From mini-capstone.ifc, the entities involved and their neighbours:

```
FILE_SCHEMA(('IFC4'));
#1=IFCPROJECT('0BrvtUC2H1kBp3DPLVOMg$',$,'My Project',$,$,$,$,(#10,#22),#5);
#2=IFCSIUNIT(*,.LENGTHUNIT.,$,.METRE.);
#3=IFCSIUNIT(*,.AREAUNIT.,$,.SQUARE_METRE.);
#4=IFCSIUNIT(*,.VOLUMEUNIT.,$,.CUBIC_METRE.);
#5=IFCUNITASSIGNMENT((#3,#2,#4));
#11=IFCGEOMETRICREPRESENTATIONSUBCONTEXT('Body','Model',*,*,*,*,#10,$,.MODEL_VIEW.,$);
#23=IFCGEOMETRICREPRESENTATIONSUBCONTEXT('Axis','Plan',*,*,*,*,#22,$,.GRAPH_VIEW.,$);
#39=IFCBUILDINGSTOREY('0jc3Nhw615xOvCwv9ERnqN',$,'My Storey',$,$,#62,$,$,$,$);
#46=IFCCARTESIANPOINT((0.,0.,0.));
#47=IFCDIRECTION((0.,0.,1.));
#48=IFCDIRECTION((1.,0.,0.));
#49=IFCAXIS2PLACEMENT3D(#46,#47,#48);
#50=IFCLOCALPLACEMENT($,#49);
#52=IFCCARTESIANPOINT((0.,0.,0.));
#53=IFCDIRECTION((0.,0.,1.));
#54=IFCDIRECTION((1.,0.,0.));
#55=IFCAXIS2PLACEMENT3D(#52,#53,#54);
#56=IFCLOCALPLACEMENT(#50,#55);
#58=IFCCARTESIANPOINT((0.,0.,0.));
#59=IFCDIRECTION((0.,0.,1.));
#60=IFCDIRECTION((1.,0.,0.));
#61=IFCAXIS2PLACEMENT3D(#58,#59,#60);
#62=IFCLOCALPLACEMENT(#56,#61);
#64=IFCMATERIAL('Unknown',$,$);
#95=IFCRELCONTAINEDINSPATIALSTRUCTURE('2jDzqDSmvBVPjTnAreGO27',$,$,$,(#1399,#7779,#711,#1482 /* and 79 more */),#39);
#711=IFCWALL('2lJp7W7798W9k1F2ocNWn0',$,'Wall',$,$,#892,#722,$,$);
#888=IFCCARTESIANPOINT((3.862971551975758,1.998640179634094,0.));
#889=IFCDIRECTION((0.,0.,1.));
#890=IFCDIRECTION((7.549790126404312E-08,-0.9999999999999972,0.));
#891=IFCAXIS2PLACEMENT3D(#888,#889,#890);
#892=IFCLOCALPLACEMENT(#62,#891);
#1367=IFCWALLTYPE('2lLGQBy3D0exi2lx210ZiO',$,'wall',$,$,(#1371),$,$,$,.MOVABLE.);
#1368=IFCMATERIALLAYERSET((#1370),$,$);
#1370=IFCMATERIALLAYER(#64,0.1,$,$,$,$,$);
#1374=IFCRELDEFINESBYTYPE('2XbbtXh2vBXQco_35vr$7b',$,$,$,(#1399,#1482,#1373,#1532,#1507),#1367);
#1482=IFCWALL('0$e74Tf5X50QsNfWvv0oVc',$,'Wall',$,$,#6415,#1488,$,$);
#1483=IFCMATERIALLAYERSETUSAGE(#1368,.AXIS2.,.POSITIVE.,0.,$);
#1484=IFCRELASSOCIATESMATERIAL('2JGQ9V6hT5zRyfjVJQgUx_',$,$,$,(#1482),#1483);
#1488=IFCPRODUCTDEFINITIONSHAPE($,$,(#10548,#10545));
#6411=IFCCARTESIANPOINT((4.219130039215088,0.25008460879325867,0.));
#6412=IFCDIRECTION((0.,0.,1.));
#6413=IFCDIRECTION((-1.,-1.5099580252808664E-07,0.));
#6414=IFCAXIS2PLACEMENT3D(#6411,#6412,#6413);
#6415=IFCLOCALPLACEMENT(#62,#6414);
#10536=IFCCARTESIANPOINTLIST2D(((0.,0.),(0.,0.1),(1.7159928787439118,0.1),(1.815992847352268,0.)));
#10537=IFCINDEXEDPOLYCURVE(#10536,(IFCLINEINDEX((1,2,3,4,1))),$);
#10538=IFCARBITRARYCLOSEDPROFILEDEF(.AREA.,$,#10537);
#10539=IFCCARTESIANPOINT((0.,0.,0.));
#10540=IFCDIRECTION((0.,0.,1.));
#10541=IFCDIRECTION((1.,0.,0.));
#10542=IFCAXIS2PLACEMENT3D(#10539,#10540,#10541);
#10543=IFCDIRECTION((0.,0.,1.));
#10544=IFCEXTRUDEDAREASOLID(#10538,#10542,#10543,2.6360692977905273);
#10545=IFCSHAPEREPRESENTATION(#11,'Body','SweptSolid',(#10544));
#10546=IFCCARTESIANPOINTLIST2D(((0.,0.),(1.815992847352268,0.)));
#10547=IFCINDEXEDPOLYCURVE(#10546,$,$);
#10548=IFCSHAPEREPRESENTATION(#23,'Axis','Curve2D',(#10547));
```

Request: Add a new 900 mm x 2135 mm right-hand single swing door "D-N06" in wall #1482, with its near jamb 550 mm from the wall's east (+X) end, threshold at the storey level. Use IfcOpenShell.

```python
import numpy as np
import ifcopenshell
import ifcopenshell.api.feature
import ifcopenshell.api.geometry
import ifcopenshell.api.root
import ifcopenshell.api.spatial
import ifcopenshell.geom
import ifcopenshell.util.element
import ifcopenshell.util.placement
import ifcopenshell.util.representation
import ifcopenshell.util.shape
import ifcopenshell.util.unit

model = ifcopenshell.open("mini-capstone.ifc")
unit_scale = ifcopenshell.util.unit.calculate_unit_scale(model)
settings = ifcopenshell.geom.settings()


def volume(element):
    """Net volume in cubic metres, openings subtracted."""
    shape = ifcopenshell.geom.create_shape(settings, element)
    return ifcopenshell.util.shape.get_volume(shape.geometry)


wall = model.by_id(1482)
storey = ifcopenshell.util.element.get_container(wall, ifc_class="IfcBuildingStorey")
context = ifcopenshell.util.representation.get_context(model, "Model", "Body", "MODEL_VIEW")
before = volume(wall)

width, height, from_end, sill = 0.9, 2.135, 0.55, 0.0  # metres

# The wall runs along its own X axis, and the end named is its -X end.
wall_shape = ifcopenshell.geom.create_shape(settings, wall)
x, y, z = ifcopenshell.util.shape.get_vertices(wall_shape.geometry).T
start = x.min() + from_end
face, thickness = float(y.min()), float(y.max() - y.min())
wall_matrix = ifcopenshell.util.placement.get_local_placement(wall.ObjectPlacement)
level = ifcopenshell.util.placement.get_local_placement(storey.ObjectPlacement)[2, 3]


def in_wall(x, y):
    """Placement at x, y metres in the wall's axes, at sill height."""
    matrix = wall_matrix.copy()
    matrix[:, 3] = wall_matrix @ np.array([x / unit_scale, y / unit_scale, 0.0, 1.0])
    matrix[2, 3] = level + sill / unit_scale
    return matrix


# Opening: a box that overshoots both wall faces by 50 mm.
opening = ifcopenshell.api.root.create_entity(model, ifc_class="IfcOpeningElement", predefined_type="OPENING")
box = ifcopenshell.api.geometry.add_wall_representation(
    model, context=context, length=width, height=height, thickness=thickness + 0.1
)
ifcopenshell.api.geometry.assign_representation(model, product=opening, representation=box)
ifcopenshell.api.geometry.edit_object_placement(model, product=opening, matrix=in_wall(start, face - 0.05), is_si=False)
ifcopenshell.api.feature.add_feature(model, feature=opening, element=wall)

door = ifcopenshell.api.root.create_entity(model, ifc_class="IfcDoor", name="D-N06", predefined_type="DOOR")
door.OverallWidth, door.OverallHeight = width / unit_scale, height / unit_scale
door.OperationType = "SINGLE_SWING_RIGHT"
body = ifcopenshell.api.geometry.add_door_representation(
    model,
    context=context,
    overall_width=door.OverallWidth,
    overall_height=door.OverallHeight,
    operation_type="SINGLE_SWING_RIGHT",
    lining_properties={"LiningDepth": thickness / unit_scale, "ThresholdDepth": thickness / unit_scale},
)
ifcopenshell.api.geometry.assign_representation(model, product=door, representation=body)
ifcopenshell.api.spatial.assign_container(model, products=[door], relating_structure=storey)
ifcopenshell.api.feature.add_filling(model, opening=opening, element=door)

# The lining spans the wall, so the door starts at the wall face.
ifcopenshell.api.geometry.edit_object_placement(model, product=door, matrix=in_wall(start, face), is_si=False)

after = volume(wall)

print(f"wall volume {before:.3f} -> {after:.3f} m3")

model.write("mini-capstone-out.ifc")
```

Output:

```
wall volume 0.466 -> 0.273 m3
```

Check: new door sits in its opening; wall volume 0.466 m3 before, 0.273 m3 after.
